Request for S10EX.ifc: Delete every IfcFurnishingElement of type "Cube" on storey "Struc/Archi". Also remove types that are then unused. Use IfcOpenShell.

First a look at what the model holds.

```python
import ifcopenshell
import ifcopenshell.util.element

model = ifcopenshell.open("S10EX.ifc")
print(model.schema)
storey = next(s for s in model.by_type("IfcBuildingStorey") if s.Name == "Struc/Archi")
furniture = [e for e in ifcopenshell.util.element.get_decomposition(storey) if e.is_a("IfcFurnishingElement")]
seen = {}
for e in furniture:
    element_type = ifcopenshell.util.element.get_type(e)
    name = element_type.Name if element_type not in (None, e) else None
    seen[name] = seen.get(name, 0) + 1
for name, count in sorted(seen.items(), key=str):
    print(count, "x", name)
```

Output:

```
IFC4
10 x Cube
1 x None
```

```python
import ifcopenshell
import ifcopenshell.api.root
import ifcopenshell.util.element

model = ifcopenshell.open("S10EX.ifc")

storey = next(s for s in model.by_type("IfcBuildingStorey") if s.Name == "Struc/Archi")
furniture = [e for e in ifcopenshell.util.element.get_decomposition(storey) if e.is_a("IfcFurnishingElement")]
targets = [e for e in furniture if (t := ifcopenshell.util.element.get_type(e)) not in (None, e) and t.Name == "Cube"]
types = {ifcopenshell.util.element.get_type(e) for e in targets} - {None, *targets}

for e in targets:
    ifcopenshell.api.root.remove_product(model, product=e)
print(len(targets), "removed")

unused = [t for t in types if not ifcopenshell.util.element.get_types(t)]
for t in unused:
    ifcopenshell.api.root.remove_product(model, product=t)
print(len(unused), "unused types removed")

model.write("S10EX_rev.ifc")
```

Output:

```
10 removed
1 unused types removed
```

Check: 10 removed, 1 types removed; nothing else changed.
